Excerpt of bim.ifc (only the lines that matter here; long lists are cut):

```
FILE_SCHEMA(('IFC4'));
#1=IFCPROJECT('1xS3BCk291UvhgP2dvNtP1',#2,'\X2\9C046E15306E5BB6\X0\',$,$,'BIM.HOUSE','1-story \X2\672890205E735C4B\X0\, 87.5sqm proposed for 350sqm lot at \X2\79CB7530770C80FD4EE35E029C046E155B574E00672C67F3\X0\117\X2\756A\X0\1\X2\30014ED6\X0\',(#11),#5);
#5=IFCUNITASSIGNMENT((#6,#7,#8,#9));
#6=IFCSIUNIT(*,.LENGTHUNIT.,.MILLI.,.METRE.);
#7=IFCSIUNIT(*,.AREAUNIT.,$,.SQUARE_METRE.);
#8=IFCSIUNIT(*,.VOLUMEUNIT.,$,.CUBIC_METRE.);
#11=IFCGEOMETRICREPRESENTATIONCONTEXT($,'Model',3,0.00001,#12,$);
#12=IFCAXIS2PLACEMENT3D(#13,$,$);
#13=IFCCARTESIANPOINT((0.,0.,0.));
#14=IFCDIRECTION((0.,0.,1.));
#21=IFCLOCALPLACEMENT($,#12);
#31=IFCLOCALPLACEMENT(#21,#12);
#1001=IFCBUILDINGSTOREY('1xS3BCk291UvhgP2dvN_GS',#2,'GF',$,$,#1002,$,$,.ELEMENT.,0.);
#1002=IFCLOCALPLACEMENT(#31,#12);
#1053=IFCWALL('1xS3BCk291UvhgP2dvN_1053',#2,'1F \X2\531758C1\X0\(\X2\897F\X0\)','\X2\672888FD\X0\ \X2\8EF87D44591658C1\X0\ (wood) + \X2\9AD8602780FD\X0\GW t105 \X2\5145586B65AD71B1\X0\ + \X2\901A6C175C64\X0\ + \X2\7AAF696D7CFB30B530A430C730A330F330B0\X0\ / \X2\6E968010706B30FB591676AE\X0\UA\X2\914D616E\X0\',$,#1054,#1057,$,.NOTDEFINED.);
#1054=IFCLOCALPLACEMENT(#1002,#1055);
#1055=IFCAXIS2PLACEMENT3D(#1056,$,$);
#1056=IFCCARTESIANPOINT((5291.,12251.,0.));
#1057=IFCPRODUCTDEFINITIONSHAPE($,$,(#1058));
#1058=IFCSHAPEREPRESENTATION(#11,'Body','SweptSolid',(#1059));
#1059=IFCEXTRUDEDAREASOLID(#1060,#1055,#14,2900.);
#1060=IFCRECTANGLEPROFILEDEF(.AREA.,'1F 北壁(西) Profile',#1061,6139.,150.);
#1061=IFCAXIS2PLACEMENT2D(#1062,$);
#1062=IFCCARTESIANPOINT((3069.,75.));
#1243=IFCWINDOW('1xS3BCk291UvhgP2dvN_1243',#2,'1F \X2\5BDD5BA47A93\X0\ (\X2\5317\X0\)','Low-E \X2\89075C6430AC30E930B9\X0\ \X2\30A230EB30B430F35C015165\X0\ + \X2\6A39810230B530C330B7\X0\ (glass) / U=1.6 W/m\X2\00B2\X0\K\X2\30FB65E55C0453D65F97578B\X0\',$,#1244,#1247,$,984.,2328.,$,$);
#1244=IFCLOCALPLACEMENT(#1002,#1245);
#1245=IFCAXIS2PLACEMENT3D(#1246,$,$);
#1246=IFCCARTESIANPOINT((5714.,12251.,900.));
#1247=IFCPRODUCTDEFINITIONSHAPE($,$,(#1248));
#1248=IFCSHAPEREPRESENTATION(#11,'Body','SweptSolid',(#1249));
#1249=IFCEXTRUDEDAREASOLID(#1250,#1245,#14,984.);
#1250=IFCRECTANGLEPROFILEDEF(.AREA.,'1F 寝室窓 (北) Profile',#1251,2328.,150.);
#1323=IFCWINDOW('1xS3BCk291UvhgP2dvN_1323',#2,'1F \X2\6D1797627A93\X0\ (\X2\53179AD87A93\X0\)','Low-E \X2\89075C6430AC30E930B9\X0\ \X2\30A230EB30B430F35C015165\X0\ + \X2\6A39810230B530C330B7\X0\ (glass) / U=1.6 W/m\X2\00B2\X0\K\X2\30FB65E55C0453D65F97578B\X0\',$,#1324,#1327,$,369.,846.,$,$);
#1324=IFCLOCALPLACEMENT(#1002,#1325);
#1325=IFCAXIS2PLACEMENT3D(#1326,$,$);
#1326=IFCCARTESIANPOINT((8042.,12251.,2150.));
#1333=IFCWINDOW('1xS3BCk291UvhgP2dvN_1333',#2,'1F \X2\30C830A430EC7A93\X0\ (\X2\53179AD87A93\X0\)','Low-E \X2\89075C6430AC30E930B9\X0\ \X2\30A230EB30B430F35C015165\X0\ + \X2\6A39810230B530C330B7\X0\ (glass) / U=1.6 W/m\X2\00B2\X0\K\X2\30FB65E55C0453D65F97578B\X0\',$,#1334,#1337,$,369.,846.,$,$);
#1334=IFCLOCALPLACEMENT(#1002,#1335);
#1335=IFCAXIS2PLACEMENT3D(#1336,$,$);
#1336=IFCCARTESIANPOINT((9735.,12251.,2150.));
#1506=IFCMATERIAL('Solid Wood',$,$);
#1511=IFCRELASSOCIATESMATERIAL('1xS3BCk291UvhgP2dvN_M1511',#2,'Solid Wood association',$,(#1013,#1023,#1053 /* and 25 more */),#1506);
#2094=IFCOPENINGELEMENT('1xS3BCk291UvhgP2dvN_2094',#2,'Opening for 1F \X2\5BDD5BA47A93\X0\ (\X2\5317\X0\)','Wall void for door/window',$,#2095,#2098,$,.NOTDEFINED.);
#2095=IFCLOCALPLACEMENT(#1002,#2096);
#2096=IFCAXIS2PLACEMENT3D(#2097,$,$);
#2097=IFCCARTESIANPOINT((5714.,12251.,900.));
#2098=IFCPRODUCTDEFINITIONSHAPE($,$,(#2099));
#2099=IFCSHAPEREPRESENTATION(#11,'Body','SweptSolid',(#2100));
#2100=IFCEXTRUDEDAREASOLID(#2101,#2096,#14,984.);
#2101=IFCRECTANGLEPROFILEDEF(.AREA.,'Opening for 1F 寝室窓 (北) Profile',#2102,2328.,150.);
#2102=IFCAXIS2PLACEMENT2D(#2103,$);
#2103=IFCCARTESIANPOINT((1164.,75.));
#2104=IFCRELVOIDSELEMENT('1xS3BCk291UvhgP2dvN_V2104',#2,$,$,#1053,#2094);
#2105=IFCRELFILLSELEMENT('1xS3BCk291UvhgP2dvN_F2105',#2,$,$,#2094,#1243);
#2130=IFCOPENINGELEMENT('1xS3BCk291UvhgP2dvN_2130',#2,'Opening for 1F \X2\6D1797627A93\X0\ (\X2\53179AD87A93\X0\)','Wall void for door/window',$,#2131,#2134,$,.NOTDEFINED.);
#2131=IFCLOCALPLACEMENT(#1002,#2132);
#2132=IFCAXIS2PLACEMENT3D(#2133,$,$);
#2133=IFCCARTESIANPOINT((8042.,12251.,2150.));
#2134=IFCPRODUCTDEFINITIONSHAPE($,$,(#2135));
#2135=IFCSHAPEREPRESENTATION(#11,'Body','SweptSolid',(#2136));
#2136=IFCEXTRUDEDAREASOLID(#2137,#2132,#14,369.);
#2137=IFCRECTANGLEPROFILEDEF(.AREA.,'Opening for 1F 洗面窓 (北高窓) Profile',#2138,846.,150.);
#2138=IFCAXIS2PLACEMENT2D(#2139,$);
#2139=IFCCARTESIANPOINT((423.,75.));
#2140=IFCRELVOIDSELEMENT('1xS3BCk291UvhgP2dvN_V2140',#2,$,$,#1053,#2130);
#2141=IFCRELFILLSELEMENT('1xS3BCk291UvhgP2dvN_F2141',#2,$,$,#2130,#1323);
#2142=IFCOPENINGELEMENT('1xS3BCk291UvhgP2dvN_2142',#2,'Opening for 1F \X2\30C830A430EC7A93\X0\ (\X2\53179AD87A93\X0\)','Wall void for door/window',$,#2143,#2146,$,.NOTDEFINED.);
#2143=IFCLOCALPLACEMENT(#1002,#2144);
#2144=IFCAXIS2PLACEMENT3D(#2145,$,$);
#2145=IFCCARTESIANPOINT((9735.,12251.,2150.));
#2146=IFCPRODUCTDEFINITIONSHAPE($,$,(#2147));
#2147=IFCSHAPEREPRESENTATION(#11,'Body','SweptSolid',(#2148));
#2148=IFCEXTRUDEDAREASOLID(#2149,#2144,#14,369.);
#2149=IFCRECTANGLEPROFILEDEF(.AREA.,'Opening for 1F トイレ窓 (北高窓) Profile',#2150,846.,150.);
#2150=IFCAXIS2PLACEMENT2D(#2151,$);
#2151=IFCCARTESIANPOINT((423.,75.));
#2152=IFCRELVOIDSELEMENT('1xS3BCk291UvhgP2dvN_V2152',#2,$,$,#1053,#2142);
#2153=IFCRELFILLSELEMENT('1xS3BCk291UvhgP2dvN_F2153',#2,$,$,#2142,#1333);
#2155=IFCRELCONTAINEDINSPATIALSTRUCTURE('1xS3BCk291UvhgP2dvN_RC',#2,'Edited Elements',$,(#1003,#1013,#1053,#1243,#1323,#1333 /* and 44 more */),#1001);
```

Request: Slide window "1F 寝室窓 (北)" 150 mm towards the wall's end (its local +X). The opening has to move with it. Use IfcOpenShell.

```python
import ifcopenshell
import ifcopenshell.api.geometry
import ifcopenshell.util.placement
import ifcopenshell.util.unit

model = ifcopenshell.open("bim.ifc")
unit_scale = ifcopenshell.util.unit.calculate_unit_scale(model)

window = model.by_guid("1xS3BCk291UvhgP2dvN_1243")
opening = window.FillsVoids[0].RelatingOpeningElement
wall = opening.VoidsElements[0].RelatingBuildingElement

wall_matrix = ifcopenshell.util.placement.get_local_placement(wall.ObjectPlacement)
shift = wall_matrix[:3, 0] * 0.15 / unit_scale
before = ifcopenshell.util.placement.get_local_placement(window.ObjectPlacement)[:3, 3].copy()

# The window is not placed relative to its opening, so move both.
for product in (opening, window):
    matrix = ifcopenshell.util.placement.get_local_placement(product.ObjectPlacement)
    matrix[:3, 3] += shift
    ifcopenshell.api.geometry.edit_object_placement(model, product=product, matrix=matrix, is_si=False)

after = ifcopenshell.util.placement.get_local_placement(window.ObjectPlacement)[:3, 3]
print("window moved by", (after - before).round(3) + 0.0)

model.write("bim_v2.ifc")
```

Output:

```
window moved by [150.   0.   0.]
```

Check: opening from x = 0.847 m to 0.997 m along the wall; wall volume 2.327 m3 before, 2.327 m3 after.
